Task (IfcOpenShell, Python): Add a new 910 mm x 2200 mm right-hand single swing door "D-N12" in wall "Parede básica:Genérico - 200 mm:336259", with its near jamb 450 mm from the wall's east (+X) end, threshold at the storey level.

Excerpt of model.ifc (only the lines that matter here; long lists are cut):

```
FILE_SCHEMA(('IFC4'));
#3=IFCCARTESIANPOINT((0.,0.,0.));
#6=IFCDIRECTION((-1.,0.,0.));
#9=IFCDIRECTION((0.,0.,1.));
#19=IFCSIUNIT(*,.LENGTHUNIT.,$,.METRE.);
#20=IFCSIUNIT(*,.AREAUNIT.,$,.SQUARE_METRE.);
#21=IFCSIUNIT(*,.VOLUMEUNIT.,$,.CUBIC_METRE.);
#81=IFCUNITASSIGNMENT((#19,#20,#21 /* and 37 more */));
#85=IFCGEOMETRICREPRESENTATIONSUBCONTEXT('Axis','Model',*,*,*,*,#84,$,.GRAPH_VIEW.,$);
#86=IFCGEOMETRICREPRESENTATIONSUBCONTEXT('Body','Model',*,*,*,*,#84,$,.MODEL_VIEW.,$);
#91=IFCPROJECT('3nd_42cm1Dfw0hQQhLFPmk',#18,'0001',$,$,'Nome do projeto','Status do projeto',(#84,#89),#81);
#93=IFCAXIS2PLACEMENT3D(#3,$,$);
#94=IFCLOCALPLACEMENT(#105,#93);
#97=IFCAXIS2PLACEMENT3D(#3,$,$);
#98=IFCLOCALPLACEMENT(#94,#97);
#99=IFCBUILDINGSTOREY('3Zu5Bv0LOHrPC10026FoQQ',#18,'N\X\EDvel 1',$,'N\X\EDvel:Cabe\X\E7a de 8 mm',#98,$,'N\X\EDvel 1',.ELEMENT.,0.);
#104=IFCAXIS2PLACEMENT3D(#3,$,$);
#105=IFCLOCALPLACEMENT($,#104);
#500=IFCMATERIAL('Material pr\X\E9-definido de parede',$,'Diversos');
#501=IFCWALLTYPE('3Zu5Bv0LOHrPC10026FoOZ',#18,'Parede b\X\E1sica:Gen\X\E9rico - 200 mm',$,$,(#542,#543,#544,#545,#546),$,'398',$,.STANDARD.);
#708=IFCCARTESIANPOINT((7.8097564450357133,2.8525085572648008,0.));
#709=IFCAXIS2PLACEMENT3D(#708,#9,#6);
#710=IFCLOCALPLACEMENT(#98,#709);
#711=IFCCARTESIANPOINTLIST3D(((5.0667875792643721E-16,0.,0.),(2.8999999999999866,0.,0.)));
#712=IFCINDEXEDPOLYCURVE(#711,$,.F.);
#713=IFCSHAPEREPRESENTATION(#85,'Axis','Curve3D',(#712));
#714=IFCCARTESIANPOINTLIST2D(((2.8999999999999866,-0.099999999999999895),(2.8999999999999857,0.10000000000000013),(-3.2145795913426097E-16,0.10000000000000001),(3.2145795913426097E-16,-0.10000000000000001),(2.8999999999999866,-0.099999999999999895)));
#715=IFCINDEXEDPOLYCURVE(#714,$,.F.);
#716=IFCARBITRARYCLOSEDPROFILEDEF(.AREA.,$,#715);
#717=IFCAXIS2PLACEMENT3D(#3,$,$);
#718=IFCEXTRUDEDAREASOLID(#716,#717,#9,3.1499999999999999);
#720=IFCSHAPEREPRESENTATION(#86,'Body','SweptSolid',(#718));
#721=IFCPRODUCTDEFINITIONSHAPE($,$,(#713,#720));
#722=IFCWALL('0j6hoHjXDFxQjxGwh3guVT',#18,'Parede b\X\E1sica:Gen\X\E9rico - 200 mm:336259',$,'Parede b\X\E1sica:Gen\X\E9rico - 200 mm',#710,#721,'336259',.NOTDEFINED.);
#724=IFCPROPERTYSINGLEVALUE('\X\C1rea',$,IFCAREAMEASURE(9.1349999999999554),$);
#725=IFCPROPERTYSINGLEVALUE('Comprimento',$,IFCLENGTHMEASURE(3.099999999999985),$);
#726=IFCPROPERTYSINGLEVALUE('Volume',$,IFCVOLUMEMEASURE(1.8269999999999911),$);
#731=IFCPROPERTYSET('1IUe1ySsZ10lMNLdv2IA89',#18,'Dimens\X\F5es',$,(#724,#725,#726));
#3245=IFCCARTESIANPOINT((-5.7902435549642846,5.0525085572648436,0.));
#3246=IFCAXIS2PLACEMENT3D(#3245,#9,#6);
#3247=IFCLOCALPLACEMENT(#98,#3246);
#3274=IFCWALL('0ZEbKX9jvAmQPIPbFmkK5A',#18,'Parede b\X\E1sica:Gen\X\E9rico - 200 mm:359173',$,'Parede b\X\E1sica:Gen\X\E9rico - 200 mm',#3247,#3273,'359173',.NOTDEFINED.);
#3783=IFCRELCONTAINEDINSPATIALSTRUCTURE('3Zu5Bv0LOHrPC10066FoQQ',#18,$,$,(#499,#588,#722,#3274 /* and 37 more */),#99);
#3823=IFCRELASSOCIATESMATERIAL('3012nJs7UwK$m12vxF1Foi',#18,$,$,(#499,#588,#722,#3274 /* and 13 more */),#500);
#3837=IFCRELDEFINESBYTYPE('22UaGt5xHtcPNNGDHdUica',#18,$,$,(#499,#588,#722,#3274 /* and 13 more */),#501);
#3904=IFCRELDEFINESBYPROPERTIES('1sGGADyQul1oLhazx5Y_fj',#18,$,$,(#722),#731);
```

```python
import numpy as np
import ifcopenshell
import ifcopenshell.api.feature
import ifcopenshell.api.geometry
import ifcopenshell.api.pset
import ifcopenshell.api.root
import ifcopenshell.api.spatial
import ifcopenshell.geom
import ifcopenshell.util.element
import ifcopenshell.util.placement
import ifcopenshell.util.representation
import ifcopenshell.util.shape
import ifcopenshell.util.unit

model = ifcopenshell.open("model.ifc")
unit_scale = ifcopenshell.util.unit.calculate_unit_scale(model)
area_scale = ifcopenshell.util.unit.calculate_unit_scale(model, "AREAUNIT")
volume_scale = ifcopenshell.util.unit.calculate_unit_scale(model, "VOLUMEUNIT")
settings = ifcopenshell.geom.settings()


def volume(element):
    """Net volume in cubic metres, openings subtracted."""
    shape = ifcopenshell.geom.create_shape(settings, element)
    return ifcopenshell.util.shape.get_volume(shape.geometry)


wall = model.by_guid("0j6hoHjXDFxQjxGwh3guVT")
storey = ifcopenshell.util.element.get_container(wall, ifc_class="IfcBuildingStorey")
context = ifcopenshell.util.representation.get_context(model, "Model", "Body", "MODEL_VIEW")
before = volume(wall)

width, height, from_end, sill = 0.91, 2.2, 0.45, 0.0  # metres

# The wall runs along its own X axis, and the end named is its -X end.
wall_shape = ifcopenshell.geom.create_shape(settings, wall)
x, y, z = ifcopenshell.util.shape.get_vertices(wall_shape.geometry).T
start = x.min() + from_end
face, thickness = float(y.min()), float(y.max() - y.min())
wall_matrix = ifcopenshell.util.placement.get_local_placement(wall.ObjectPlacement)
level = ifcopenshell.util.placement.get_local_placement(storey.ObjectPlacement)[2, 3]


def in_wall(x, y):
    """Placement at x, y metres in the wall's axes, at sill height."""
    matrix = wall_matrix.copy()
    matrix[:, 3] = wall_matrix @ np.array([x / unit_scale, y / unit_scale, 0.0, 1.0])
    matrix[2, 3] = level + sill / unit_scale
    return matrix


# Opening: a box that overshoots both wall faces by 50 mm.
opening = ifcopenshell.api.root.create_entity(model, ifc_class="IfcOpeningElement", predefined_type="OPENING")
box = ifcopenshell.api.geometry.add_wall_representation(
    model, context=context, length=width, height=height, thickness=thickness + 0.1
)
ifcopenshell.api.geometry.assign_representation(model, product=opening, representation=box)
ifcopenshell.api.geometry.edit_object_placement(model, product=opening, matrix=in_wall(start, face - 0.05), is_si=False)
ifcopenshell.api.feature.add_feature(model, feature=opening, element=wall)

door = ifcopenshell.api.root.create_entity(model, ifc_class="IfcDoor", name="D-N12", predefined_type="DOOR")
door.OverallWidth, door.OverallHeight = width / unit_scale, height / unit_scale
door.OperationType = "SINGLE_SWING_RIGHT"
body = ifcopenshell.api.geometry.add_door_representation(
    model,
    context=context,
    overall_width=door.OverallWidth,
    overall_height=door.OverallHeight,
    operation_type="SINGLE_SWING_RIGHT",
    lining_properties={"LiningDepth": thickness / unit_scale, "ThresholdDepth": thickness / unit_scale},
)
ifcopenshell.api.geometry.assign_representation(model, product=door, representation=body)
ifcopenshell.api.spatial.assign_container(model, products=[door], relating_structure=storey)
ifcopenshell.api.feature.add_filling(model, opening=opening, element=door)

# The lining spans the wall, so the door starts at the wall face.
ifcopenshell.api.geometry.edit_object_placement(model, product=door, matrix=in_wall(start, face), is_si=False)

after = volume(wall)

# Update the wall's stored quantities.
pset = model.by_id(ifcopenshell.util.element.get_pset(wall, "Dimensões", should_inherit=False)["id"])
ifcopenshell.api.pset.edit_pset(model, pset=pset, properties={
    "Área": model.create_entity("IfcAreaMeasure", after / thickness / area_scale),
    "Volume": model.create_entity("IfcVolumeMeasure", after / volume_scale),
})

print(f"wall volume {before:.3f} -> {after:.3f} m3")

model.write("model_v2.ifc")
```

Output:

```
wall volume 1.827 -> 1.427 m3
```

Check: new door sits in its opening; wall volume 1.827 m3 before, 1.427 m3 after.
